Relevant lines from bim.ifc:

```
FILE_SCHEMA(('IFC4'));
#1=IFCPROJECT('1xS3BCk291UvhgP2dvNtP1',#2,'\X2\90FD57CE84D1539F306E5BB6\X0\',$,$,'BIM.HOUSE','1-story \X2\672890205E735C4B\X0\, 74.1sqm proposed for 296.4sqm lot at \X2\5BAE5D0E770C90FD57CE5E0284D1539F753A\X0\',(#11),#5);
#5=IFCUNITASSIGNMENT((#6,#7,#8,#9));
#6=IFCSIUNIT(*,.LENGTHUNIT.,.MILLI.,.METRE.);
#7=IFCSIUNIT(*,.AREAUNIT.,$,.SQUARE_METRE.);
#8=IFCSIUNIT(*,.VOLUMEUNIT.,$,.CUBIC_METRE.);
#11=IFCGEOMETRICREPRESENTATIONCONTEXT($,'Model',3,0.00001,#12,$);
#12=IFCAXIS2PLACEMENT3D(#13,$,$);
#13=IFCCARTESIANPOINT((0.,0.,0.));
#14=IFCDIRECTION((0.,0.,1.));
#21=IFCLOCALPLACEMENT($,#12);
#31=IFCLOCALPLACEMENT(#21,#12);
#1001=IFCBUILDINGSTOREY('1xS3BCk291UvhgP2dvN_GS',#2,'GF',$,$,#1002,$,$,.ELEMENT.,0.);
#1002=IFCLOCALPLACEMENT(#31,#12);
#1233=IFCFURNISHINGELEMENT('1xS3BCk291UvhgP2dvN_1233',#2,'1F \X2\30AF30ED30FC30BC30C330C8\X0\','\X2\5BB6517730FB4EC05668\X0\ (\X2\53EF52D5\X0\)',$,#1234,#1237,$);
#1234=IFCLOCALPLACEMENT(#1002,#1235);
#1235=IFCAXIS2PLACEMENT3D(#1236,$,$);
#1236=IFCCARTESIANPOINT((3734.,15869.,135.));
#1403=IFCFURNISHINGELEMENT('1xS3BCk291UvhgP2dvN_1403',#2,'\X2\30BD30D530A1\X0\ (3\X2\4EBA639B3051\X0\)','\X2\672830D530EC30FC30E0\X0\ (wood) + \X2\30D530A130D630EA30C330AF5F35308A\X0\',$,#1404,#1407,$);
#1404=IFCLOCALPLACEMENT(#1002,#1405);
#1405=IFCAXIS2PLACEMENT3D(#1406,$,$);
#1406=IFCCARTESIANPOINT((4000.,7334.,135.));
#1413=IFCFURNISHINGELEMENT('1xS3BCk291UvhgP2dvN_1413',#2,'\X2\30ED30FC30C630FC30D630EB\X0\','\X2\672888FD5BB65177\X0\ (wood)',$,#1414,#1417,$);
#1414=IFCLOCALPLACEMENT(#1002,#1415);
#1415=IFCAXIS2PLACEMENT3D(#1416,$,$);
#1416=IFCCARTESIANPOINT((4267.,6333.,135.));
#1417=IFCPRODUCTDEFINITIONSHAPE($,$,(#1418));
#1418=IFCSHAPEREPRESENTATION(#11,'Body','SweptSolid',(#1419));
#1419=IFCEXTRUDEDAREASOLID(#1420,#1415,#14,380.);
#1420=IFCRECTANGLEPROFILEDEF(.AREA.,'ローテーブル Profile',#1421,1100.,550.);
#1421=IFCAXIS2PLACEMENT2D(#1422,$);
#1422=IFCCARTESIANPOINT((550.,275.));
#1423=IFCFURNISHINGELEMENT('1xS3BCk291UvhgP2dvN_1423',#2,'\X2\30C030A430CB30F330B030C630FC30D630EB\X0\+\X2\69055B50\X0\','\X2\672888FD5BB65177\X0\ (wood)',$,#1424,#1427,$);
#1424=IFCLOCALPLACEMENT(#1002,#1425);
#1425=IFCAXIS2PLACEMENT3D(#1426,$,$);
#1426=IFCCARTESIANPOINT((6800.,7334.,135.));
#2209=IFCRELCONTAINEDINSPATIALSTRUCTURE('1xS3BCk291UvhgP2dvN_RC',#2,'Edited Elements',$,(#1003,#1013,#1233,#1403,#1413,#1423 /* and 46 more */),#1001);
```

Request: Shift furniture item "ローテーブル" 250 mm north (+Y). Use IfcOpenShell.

```python
import ifcopenshell
import ifcopenshell.api.geometry
import ifcopenshell.util.placement

model = ifcopenshell.open("bim.ifc")

item = model.by_guid("1xS3BCk291UvhgP2dvN_1413")
matrix = ifcopenshell.util.placement.get_local_placement(item.ObjectPlacement)
matrix[1, 3] += 250.0
ifcopenshell.api.geometry.edit_object_placement(model, product=item, matrix=matrix, is_si=False)

print(ifcopenshell.util.placement.get_local_placement(item.ObjectPlacement).round(3) + 0.0)

model.write("bim_updated.ifc")
```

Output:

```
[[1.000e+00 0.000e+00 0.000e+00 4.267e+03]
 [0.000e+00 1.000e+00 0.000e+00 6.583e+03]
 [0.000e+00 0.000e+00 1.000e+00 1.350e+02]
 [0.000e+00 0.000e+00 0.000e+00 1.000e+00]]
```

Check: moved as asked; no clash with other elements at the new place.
